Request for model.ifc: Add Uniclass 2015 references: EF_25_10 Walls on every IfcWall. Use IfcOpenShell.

First a look at what the model holds.

```python
import ifcopenshell

model = ifcopenshell.open("model.ifc")
print(model.schema)
print("classifications:", [c.Name for c in model.by_type("IfcClassification")])
for ifc_class in ("IfcDoor", "IfcRoof", "IfcStair", "IfcWall", "IfcWindow"):
    print(ifc_class, len(model.by_type(ifc_class)))
```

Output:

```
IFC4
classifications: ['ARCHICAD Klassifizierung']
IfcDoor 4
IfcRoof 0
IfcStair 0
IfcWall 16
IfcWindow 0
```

```python
import ifcopenshell
import ifcopenshell.api.classification

model = ifcopenshell.open("model.ifc")

system = ifcopenshell.api.classification.add_classification(model, classification="Uniclass 2015")

codes = {
    "IfcWall": ("EF_25_10", "Walls"),
}
for ifc_class, (code, name) in codes.items():
    products = model.by_type(ifc_class)
    ifcopenshell.api.classification.add_reference(
        model, products=products, classification=system, identification=code, name=name
    )
    print(code, len(products))

model.write("model_rev.ifc")
```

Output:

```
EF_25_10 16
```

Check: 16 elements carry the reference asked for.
